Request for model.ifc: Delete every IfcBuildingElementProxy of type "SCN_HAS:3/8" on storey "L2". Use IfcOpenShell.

First a look at what the model holds.

```python
import ifcopenshell
import ifcopenshell.util.element

model = ifcopenshell.open("model.ifc")
print(model.schema)
storey = next(s for s in model.by_type("IfcBuildingStorey") if s.Name == "L2")
proxies = [e for e in ifcopenshell.util.element.get_decomposition(storey) if e.is_a("IfcBuildingElementProxy")]
seen = {}
for e in proxies:
    element_type = ifcopenshell.util.element.get_type(e)
    name = element_type.Name if element_type not in (None, e) else None
    seen[name] = seen.get(name, 0) + 1
for name, count in sorted(seen.items(), key=str):
    print(count, "x", name)
```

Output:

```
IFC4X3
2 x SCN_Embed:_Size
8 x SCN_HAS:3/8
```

```python
import ifcopenshell
import ifcopenshell.api.root
import ifcopenshell.util.element

model = ifcopenshell.open("model.ifc")

storey = next(s for s in model.by_type("IfcBuildingStorey") if s.Name == "L2")
proxies = [e for e in ifcopenshell.util.element.get_decomposition(storey) if e.is_a("IfcBuildingElementProxy")]
targets = [e for e in proxies if (t := ifcopenshell.util.element.get_type(e)) not in (None, e) and t.Name == "SCN_HAS:3/8"]

for e in targets:
    ifcopenshell.api.root.remove_product(model, product=e)
print(len(targets), "removed")

model.write("model_rev.ifc")
```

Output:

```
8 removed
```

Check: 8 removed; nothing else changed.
